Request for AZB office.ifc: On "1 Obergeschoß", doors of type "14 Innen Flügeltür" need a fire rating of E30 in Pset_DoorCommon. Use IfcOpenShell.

First a look at what the model holds.

```python
import ifcopenshell
import ifcopenshell.util.element

model = ifcopenshell.open("AZB office.ifc")
print(model.schema)
storey = next(s for s in model.by_type("IfcBuildingStorey") if s.Name == "1 Obergeschoß")
doors = [e for e in ifcopenshell.util.element.get_decomposition(storey) if e.is_a("IfcDoor")]
seen = {}
for e in doors:
    element_type = ifcopenshell.util.element.get_type(e)
    key = (element_type.Name if element_type != e and element_type else None, ifcopenshell.util.element.get_pset(e, "Pset_DoorCommon", "FireRating"))
    seen[key] = seen.get(key, 0) + 1
for (name, value), count in sorted(seen.items(), key=str):
    print(count, "x", name, "|", value)
```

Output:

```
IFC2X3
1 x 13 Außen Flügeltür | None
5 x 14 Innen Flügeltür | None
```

```python
import ifcopenshell
import ifcopenshell.api.pset
import ifcopenshell.util.element

model = ifcopenshell.open("AZB office.ifc")

storey = next(s for s in model.by_type("IfcBuildingStorey") if s.Name == "1 Obergeschoß")
doors = [e for e in ifcopenshell.util.element.get_decomposition(storey) if e.is_a("IfcDoor")]

count = 0
for e in doors:
    element_type = ifcopenshell.util.element.get_type(e)
    if element_type in (None, e) or element_type.Name != "14 Innen Flügeltür":
        continue
    # add_pset returns the element's existing set when there is one.
    pset = ifcopenshell.api.pset.add_pset(model, product=e, name="Pset_DoorCommon")
    ifcopenshell.api.pset.edit_pset(model, pset=pset, properties={"FireRating": "E30"})
    count += 1

print(count, "doors updated")

model.write("AZB office_rev.ifc")
```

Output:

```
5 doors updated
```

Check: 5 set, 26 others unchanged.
